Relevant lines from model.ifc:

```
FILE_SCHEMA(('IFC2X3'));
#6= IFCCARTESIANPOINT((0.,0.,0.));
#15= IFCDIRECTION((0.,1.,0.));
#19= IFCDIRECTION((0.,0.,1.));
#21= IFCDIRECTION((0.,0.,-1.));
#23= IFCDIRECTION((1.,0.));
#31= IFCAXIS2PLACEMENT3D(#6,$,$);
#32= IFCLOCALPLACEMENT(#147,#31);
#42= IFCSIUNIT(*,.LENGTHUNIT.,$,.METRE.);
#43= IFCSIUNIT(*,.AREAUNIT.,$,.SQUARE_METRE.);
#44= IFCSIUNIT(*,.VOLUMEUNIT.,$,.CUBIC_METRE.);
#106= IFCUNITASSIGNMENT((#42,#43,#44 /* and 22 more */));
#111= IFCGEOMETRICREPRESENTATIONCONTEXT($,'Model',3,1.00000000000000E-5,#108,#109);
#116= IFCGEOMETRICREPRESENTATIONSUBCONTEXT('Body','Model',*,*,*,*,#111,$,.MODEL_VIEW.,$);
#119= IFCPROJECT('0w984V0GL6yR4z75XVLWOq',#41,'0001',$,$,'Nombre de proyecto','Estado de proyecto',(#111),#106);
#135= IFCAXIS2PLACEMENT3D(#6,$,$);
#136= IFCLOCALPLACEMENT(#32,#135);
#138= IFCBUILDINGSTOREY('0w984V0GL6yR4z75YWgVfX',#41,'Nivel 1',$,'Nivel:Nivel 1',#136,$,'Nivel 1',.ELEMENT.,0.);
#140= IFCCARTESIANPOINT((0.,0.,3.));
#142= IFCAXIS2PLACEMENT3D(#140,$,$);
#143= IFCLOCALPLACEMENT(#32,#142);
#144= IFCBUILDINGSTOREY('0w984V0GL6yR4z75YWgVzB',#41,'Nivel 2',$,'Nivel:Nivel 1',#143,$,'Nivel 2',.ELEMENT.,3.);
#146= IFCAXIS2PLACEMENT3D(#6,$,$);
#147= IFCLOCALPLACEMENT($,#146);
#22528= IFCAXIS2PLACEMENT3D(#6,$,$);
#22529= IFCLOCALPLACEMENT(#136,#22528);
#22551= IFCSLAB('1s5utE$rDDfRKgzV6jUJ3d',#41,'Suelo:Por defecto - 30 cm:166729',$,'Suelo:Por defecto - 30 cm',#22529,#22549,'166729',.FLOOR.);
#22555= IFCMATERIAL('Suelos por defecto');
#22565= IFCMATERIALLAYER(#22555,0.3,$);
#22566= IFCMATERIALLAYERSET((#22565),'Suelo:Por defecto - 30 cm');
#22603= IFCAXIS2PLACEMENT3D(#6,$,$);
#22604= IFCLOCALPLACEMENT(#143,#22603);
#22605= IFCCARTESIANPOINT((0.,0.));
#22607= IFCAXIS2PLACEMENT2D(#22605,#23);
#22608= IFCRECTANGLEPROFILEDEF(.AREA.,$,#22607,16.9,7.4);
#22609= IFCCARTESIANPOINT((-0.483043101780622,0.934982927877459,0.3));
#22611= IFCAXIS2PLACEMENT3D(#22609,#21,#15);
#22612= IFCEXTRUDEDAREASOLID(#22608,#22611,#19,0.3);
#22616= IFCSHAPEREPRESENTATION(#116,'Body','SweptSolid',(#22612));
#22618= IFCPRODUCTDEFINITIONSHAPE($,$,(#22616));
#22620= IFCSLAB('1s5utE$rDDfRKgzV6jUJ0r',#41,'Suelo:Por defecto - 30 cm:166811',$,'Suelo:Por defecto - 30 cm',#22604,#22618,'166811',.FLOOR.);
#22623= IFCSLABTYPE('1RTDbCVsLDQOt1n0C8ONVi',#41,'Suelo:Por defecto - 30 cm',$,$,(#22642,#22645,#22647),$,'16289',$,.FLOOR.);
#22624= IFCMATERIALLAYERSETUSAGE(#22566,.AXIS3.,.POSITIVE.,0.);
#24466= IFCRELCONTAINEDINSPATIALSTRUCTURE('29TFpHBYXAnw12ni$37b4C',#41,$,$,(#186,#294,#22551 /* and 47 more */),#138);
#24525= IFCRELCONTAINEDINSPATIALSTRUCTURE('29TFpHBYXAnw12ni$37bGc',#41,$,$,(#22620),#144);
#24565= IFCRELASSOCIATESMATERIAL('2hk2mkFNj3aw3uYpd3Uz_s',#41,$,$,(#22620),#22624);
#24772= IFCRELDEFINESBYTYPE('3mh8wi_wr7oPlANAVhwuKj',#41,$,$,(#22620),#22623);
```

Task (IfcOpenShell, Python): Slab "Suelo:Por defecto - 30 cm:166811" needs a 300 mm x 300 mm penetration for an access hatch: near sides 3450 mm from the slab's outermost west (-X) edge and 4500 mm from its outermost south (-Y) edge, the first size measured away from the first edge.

```python
import numpy as np
import ifcopenshell
import ifcopenshell.api.feature
import ifcopenshell.api.geometry
import ifcopenshell.api.root
import ifcopenshell.geom
import ifcopenshell.util.placement
import ifcopenshell.util.representation
import ifcopenshell.util.shape
import ifcopenshell.util.unit

model = ifcopenshell.open("model.ifc")
unit_scale = ifcopenshell.util.unit.calculate_unit_scale(model)
settings = ifcopenshell.geom.settings()


def volume(element):
    """Net volume in cubic metres, openings subtracted."""
    shape = ifcopenshell.geom.create_shape(settings, element)
    return ifcopenshell.util.shape.get_volume(shape.geometry)


slab = model.by_guid("1s5utE$rDDfRKgzV6jUJ0r")
before = volume(slab)

# Extent in the slab's own axes, in metres. The edges named are its -X and -Y sides.
slab_shape = ifcopenshell.geom.create_shape(settings, slab)
vertices = ifcopenshell.util.shape.get_vertices(slab_shape.geometry)
x_min, y_min, bottom = vertices.min(axis=0)
top = vertices[:, 2].max()

opening = ifcopenshell.api.root.create_entity(model, ifc_class="IfcOpeningElement", name="Access hatch opening")
context = ifcopenshell.util.representation.get_context(model, "Model", "Body", "MODEL_VIEW")
width, depth = 0.3, 0.3
outline = [(0.0, 0.0), (width, 0.0), (width, depth), (0.0, depth), (0.0, 0.0)]
# Overshoot both faces by 50 mm so the cut is clean.
shape = ifcopenshell.api.geometry.add_slab_representation(
    model, context=context, depth=top - bottom + 0.1, polyline=outline
)
ifcopenshell.api.geometry.assign_representation(model, product=opening, representation=shape)

matrix = ifcopenshell.util.placement.get_local_placement(slab.ObjectPlacement)
matrix[:, 3] = matrix @ np.append(np.array([x_min + 3.45, y_min + 4.5, bottom - 0.05]) / unit_scale, 1.0)
ifcopenshell.api.geometry.edit_object_placement(model, product=opening, matrix=matrix, is_si=False)
ifcopenshell.api.feature.add_feature(model, feature=opening, element=slab)

after = volume(slab)

print(f"slab volume {before:.3f} -> {after:.3f} m3")

model.write("model_updated.ifc")
```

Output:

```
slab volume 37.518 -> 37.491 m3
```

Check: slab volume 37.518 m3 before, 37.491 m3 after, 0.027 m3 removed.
